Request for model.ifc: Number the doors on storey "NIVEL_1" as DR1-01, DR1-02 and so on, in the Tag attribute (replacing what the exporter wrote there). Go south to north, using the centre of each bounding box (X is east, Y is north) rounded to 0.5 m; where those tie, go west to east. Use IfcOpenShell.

First a look at what the model holds.

```python
import ifcopenshell
import ifcopenshell.util.element
import ifcopenshell.util.placement

model = ifcopenshell.open("model.ifc")
print(model.schema)
storey = next(s for s in model.by_type("IfcBuildingStorey") if s.Name == "NIVEL_1")
doors = [e for e in ifcopenshell.util.element.get_decomposition(storey) if e.is_a("IfcDoor")]
for e in sorted(doors, key=lambda e: e.id()):
    origin = ifcopenshell.util.placement.get_local_placement(e.ObjectPlacement)[:3, 3]
    print(e.id(), e.Tag, e.Name, origin.round(2) + 0.0, sep=" | ")
```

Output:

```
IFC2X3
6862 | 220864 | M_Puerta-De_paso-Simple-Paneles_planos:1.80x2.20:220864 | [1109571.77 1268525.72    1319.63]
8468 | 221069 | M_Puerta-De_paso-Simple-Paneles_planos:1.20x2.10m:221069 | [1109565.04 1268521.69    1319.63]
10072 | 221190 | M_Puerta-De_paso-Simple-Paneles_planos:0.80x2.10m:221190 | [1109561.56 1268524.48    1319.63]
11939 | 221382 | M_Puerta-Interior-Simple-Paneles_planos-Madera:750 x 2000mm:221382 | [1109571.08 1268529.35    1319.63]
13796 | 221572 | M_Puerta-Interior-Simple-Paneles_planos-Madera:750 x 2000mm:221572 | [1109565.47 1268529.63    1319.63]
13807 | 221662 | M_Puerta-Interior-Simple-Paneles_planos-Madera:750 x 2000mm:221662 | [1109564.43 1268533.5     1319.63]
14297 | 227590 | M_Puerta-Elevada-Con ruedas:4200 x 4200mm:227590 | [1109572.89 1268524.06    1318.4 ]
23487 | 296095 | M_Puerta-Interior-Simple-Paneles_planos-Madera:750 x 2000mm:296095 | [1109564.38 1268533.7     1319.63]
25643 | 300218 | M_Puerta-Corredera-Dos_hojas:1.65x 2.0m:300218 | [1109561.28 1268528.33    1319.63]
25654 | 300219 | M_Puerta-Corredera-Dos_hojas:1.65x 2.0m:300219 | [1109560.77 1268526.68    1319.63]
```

```python
import ifcopenshell
import ifcopenshell.geom
import ifcopenshell.util.element
import ifcopenshell.util.shape

model = ifcopenshell.open("model.ifc")
settings = ifcopenshell.geom.settings()
settings.set("use-world-coords", True)


def centre(element):
    shape = ifcopenshell.geom.create_shape(settings, element)
    return ifcopenshell.util.shape.get_bbox_centroid(shape.geometry)


storey = next(s for s in model.by_type("IfcBuildingStorey") if s.Name == "NIVEL_1")
doors = [e for e in ifcopenshell.util.element.get_decomposition(storey) if e.is_a("IfcDoor")]

# Insertion points can sit at a corner or the storey origin, so sort by the geometry (in metres).
centres = {e: centre(e) for e in doors}
doors.sort(key=lambda e: (round(centres[e][1] / 0.5), centres[e][0]))

for i, e in enumerate(doors, start=1):
    number = f"DR1-{i:02d}"
    e.Tag = number
    print(e.id(), number)

model.write("model_rev.ifc")
```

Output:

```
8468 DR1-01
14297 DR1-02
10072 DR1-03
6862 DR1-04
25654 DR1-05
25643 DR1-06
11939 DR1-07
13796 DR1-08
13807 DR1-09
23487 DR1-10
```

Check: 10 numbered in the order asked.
